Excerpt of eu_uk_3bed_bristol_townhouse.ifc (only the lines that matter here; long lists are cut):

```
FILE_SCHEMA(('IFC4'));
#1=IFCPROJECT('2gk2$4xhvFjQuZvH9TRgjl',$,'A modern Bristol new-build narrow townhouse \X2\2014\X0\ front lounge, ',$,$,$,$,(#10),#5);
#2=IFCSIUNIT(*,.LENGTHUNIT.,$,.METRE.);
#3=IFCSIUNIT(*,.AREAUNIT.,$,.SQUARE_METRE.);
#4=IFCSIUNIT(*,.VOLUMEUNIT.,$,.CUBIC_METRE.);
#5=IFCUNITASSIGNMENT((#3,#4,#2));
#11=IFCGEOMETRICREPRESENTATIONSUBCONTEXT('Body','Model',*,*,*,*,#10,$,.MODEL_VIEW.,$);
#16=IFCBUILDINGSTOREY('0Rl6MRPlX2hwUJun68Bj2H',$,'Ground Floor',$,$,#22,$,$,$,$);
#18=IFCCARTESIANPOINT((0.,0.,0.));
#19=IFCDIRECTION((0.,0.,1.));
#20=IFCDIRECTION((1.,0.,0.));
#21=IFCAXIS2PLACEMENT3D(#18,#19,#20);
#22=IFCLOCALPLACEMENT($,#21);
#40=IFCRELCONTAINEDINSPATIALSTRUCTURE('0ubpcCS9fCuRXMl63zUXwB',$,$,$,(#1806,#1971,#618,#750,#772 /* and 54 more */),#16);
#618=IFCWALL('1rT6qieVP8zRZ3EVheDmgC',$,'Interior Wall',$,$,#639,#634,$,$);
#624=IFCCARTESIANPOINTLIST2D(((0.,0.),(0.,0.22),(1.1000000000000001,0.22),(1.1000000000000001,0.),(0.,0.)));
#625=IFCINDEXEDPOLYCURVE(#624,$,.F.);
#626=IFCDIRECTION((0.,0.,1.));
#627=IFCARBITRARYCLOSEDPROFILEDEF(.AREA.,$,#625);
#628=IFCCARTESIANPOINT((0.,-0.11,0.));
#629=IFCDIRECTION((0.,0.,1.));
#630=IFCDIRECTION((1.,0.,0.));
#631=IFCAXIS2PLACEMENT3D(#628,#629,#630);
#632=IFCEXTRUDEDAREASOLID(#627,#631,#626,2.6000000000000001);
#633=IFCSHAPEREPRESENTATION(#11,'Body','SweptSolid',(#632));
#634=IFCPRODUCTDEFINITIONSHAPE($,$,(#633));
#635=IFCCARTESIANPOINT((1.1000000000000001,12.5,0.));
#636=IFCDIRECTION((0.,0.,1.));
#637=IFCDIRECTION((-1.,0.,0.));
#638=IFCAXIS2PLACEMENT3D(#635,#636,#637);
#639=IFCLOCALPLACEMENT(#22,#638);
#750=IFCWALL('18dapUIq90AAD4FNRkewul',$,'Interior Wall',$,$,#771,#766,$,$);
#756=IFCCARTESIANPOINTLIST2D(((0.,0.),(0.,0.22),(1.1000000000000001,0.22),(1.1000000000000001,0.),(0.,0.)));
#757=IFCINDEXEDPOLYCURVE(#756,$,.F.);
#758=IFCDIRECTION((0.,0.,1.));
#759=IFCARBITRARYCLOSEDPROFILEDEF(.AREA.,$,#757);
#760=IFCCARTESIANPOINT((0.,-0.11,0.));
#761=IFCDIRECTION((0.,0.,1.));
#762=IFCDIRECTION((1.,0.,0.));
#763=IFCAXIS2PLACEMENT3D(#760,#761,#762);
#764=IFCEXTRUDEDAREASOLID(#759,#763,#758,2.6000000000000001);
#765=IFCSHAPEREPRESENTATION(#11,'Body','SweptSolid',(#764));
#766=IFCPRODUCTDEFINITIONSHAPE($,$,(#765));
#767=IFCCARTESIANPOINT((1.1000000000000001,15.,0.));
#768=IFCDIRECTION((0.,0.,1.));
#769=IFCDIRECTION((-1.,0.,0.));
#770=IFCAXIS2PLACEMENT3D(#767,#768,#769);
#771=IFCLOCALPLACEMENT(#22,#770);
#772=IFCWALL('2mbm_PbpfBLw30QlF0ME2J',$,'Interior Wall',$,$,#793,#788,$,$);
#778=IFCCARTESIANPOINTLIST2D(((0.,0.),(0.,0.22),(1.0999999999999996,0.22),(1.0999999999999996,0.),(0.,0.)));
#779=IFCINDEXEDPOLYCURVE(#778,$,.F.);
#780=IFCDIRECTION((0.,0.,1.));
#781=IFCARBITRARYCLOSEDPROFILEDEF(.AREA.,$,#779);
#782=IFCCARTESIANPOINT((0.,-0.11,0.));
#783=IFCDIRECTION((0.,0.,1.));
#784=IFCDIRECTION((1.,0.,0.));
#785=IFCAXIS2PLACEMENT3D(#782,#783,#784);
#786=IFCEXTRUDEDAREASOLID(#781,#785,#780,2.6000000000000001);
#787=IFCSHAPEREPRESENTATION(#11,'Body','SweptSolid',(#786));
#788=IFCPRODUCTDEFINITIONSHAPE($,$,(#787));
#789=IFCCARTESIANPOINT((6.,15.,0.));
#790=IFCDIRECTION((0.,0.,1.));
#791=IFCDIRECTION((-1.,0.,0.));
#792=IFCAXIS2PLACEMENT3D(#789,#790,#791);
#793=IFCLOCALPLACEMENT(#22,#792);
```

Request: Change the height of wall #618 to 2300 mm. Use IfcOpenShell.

```python
import ifcopenshell
import ifcopenshell.geom
import ifcopenshell.util.representation
import ifcopenshell.util.shape
import ifcopenshell.util.unit

model = ifcopenshell.open("eu_uk_3bed_bristol_townhouse.ifc")
unit_scale = ifcopenshell.util.unit.calculate_unit_scale(model)
settings = ifcopenshell.geom.settings()


def volume(element):
    """Net volume in cubic metres, openings subtracted."""
    shape = ifcopenshell.geom.create_shape(settings, element)
    return ifcopenshell.util.shape.get_volume(shape.geometry)


wall = model.by_guid("1rT6qieVP8zRZ3EVheDmgC")
before = volume(wall)

body = ifcopenshell.util.representation.get_representation(wall, "Model", "Body")
solid = body.Items[0]
old_height = solid.Depth
solid.Depth = 2.3 / unit_scale
after = volume(wall)

print(f"height {old_height:g} -> {solid.Depth:g}, volume {before:.3f} -> {after:.3f} m3")

model.write("eu_uk_3bed_bristol_townhouse-out.ifc")
```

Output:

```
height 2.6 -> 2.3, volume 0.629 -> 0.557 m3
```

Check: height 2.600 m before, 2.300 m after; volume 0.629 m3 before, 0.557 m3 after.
